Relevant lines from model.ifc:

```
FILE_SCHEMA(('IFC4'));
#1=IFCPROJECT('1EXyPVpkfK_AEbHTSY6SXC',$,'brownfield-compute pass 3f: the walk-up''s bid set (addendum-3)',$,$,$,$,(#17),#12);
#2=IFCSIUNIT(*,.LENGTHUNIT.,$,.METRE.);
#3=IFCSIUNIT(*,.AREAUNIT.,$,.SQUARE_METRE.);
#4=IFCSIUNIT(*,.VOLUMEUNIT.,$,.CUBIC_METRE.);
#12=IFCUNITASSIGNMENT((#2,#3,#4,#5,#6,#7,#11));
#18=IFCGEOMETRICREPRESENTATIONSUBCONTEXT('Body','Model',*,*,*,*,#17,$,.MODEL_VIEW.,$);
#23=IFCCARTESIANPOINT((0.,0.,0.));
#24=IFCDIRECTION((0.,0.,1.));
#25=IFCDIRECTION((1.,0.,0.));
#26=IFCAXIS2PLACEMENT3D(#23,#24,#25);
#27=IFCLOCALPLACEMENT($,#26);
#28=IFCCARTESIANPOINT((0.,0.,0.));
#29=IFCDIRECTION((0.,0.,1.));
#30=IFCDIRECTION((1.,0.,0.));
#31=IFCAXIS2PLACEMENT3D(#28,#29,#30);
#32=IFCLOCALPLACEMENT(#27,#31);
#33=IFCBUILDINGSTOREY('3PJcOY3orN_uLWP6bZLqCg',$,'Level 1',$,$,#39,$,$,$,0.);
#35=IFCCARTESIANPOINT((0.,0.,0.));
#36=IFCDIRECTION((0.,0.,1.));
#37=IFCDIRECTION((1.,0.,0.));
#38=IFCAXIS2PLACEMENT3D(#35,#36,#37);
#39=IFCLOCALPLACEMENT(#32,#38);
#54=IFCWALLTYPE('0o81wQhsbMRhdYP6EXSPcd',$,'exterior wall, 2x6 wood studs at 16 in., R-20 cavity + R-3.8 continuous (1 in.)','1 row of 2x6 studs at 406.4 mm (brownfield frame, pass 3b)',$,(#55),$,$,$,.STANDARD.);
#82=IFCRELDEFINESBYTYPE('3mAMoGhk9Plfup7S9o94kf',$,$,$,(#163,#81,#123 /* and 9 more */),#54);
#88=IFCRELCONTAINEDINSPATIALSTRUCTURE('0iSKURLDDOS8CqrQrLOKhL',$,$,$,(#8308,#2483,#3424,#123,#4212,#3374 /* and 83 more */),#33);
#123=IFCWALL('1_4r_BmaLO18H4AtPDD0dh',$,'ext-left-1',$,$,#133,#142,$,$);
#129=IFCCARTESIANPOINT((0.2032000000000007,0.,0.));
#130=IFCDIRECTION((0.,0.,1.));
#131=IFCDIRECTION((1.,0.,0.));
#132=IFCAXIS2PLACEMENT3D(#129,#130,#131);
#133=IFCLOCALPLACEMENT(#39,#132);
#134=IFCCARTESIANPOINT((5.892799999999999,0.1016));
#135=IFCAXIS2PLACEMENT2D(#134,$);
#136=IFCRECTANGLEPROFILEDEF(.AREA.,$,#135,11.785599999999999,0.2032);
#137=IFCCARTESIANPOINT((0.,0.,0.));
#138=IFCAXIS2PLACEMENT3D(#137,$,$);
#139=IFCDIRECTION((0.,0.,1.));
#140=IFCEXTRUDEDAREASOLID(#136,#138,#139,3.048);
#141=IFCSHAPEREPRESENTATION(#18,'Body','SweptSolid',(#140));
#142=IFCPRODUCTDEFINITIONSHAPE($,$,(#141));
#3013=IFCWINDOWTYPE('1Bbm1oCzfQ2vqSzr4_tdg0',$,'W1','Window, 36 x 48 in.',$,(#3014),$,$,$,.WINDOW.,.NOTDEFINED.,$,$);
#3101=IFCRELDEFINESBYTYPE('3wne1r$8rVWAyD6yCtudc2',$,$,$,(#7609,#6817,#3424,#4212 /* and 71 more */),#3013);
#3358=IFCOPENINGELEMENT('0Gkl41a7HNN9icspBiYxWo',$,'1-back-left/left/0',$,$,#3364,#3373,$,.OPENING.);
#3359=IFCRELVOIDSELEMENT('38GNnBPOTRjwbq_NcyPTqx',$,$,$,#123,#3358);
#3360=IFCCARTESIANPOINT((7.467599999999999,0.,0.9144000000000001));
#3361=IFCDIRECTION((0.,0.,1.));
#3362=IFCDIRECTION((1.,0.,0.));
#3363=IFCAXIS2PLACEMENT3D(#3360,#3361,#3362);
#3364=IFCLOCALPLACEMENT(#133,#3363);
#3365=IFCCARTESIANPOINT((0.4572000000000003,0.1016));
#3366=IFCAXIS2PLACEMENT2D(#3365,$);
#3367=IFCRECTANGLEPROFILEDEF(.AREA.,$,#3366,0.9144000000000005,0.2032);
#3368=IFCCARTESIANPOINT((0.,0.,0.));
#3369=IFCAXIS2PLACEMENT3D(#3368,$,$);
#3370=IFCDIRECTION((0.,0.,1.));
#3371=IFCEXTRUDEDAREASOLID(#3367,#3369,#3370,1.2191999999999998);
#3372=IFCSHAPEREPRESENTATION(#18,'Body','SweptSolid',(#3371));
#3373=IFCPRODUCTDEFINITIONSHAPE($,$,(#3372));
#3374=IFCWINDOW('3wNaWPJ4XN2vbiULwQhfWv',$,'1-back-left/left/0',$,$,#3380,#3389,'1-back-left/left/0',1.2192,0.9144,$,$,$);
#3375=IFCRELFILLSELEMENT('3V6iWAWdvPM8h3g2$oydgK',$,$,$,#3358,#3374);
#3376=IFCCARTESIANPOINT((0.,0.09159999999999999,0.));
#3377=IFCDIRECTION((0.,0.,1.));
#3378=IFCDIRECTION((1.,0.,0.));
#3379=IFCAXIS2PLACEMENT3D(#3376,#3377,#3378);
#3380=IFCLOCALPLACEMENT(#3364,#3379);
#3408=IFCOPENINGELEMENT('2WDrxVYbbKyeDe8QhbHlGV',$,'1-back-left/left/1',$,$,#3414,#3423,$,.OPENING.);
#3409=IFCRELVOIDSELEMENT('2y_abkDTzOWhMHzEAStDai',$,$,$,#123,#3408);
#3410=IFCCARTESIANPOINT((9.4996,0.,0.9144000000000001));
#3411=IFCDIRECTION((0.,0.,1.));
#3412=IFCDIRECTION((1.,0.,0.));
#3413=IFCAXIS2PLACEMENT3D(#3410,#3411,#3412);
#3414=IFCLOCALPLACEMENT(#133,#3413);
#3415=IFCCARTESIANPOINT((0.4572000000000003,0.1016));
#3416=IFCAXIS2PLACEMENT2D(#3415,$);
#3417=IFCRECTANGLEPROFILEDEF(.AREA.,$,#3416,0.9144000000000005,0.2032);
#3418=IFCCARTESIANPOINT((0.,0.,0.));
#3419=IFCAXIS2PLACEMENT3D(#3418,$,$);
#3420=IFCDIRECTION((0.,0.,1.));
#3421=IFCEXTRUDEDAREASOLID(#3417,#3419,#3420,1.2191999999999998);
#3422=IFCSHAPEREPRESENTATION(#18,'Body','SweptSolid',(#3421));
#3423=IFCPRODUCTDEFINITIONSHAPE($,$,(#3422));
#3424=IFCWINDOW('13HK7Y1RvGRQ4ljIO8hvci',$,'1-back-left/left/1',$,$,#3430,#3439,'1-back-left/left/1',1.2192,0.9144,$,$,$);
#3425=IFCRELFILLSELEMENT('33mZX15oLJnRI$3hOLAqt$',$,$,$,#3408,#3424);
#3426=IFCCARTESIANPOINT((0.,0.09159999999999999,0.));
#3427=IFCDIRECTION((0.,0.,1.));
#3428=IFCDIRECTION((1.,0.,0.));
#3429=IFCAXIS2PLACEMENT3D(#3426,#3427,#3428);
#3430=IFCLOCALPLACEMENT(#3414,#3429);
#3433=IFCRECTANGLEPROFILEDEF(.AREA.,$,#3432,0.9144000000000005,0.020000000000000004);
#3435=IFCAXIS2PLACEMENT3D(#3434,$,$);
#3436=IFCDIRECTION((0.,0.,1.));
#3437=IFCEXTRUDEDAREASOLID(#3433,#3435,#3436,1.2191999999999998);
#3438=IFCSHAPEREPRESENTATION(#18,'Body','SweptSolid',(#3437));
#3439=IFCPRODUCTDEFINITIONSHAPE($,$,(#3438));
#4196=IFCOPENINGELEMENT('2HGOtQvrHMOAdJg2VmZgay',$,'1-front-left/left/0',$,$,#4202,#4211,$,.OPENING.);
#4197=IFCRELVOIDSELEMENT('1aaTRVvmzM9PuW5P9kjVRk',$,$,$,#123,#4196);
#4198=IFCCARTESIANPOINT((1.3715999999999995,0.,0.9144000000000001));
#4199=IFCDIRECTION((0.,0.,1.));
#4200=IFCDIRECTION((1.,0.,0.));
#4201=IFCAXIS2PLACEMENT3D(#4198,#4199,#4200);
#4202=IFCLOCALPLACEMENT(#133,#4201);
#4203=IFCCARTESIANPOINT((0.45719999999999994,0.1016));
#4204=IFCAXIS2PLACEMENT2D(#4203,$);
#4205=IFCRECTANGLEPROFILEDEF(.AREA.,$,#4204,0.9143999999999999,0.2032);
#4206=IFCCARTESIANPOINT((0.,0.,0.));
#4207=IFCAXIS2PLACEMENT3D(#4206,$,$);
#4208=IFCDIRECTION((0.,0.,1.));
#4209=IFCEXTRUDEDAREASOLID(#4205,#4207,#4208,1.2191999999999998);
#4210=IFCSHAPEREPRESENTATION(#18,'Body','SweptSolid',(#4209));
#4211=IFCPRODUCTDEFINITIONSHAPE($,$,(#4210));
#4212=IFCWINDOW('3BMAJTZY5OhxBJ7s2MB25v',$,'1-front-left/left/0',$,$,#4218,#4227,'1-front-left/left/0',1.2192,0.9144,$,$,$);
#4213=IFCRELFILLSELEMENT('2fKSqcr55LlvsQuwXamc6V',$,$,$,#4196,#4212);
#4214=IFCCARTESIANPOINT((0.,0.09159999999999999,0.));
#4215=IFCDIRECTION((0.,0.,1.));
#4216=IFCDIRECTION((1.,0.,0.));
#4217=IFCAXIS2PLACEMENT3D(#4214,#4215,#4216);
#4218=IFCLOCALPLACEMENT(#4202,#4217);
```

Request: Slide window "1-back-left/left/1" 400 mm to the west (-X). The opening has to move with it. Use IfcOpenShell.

```python
import ifcopenshell
import ifcopenshell.api.geometry
import ifcopenshell.util.placement
import ifcopenshell.util.unit

model = ifcopenshell.open("model.ifc")
unit_scale = ifcopenshell.util.unit.calculate_unit_scale(model)

window = model.by_guid("13HK7Y1RvGRQ4ljIO8hvci")
opening = window.FillsVoids[0].RelatingOpeningElement
wall = opening.VoidsElements[0].RelatingBuildingElement

wall_matrix = ifcopenshell.util.placement.get_local_placement(wall.ObjectPlacement)
shift = wall_matrix[:3, 0] * -0.4 / unit_scale
before = ifcopenshell.util.placement.get_local_placement(window.ObjectPlacement)[:3, 3].copy()

# The window is placed relative to its opening, so it follows when the opening moves.
matrix = ifcopenshell.util.placement.get_local_placement(opening.ObjectPlacement)
matrix[:3, 3] += shift
ifcopenshell.api.geometry.edit_object_placement(
    model, product=opening, matrix=matrix, is_si=False, should_transform_children=True
)

after = ifcopenshell.util.placement.get_local_placement(window.ObjectPlacement)[:3, 3]
print("window moved by", (after - before).round(3) + 0.0)

model.write("model_rev.ifc")
```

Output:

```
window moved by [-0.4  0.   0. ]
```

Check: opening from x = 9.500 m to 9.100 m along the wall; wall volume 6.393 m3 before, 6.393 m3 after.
